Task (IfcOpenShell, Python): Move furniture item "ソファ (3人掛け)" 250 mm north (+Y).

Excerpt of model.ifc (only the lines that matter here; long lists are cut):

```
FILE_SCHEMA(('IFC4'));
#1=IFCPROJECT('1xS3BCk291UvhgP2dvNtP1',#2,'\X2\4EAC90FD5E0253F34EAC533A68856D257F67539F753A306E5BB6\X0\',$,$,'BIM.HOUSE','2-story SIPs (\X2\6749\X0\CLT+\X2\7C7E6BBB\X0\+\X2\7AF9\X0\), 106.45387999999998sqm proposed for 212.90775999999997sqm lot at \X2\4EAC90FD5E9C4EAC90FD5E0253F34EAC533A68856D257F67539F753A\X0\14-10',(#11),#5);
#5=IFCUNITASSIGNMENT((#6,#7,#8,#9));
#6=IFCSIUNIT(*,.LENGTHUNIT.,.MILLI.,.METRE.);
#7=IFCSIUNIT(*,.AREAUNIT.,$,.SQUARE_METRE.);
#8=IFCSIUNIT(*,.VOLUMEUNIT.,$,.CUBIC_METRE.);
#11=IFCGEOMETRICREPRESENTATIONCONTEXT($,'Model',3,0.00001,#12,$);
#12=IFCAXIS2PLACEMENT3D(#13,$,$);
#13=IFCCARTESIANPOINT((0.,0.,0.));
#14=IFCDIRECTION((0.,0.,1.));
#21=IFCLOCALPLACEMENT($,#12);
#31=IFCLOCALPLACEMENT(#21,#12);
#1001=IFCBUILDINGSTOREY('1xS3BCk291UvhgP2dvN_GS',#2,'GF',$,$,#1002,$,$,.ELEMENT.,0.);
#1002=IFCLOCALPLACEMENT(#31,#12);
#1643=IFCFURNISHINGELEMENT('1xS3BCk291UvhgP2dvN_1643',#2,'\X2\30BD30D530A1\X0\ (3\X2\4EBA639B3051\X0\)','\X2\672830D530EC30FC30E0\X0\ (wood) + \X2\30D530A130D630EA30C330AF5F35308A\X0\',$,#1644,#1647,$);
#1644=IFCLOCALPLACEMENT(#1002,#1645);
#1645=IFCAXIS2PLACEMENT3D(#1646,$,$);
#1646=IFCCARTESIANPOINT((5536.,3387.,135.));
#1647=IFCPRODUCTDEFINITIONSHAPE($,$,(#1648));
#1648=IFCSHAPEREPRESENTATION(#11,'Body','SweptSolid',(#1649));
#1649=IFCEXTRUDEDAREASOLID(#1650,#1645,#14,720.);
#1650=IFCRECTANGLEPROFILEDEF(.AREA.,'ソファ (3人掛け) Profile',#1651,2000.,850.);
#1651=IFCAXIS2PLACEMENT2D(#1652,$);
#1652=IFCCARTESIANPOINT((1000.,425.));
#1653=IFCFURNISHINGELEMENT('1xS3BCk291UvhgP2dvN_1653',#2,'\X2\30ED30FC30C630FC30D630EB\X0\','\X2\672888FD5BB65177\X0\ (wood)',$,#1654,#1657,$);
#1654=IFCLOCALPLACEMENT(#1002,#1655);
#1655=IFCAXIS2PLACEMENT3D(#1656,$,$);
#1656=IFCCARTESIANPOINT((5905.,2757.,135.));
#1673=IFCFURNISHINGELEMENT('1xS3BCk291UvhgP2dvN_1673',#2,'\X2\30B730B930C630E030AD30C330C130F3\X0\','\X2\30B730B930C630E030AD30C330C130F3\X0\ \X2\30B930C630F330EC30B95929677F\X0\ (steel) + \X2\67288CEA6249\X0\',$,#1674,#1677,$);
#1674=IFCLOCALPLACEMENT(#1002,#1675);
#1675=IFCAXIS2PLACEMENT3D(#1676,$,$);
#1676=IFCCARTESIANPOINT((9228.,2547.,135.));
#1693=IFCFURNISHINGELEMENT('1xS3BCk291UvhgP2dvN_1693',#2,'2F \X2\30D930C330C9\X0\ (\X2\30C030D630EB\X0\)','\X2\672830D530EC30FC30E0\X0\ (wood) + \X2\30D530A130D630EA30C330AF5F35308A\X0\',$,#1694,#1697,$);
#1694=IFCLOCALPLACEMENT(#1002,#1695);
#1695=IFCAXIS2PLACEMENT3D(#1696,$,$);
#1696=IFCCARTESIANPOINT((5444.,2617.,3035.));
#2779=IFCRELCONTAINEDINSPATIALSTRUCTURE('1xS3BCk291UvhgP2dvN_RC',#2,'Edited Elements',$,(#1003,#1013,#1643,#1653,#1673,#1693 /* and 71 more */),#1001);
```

```python
import ifcopenshell
import ifcopenshell.api.geometry
import ifcopenshell.util.placement

model = ifcopenshell.open("model.ifc")

item = model.by_id(1643)
matrix = ifcopenshell.util.placement.get_local_placement(item.ObjectPlacement)
matrix[1, 3] += 250.0
ifcopenshell.api.geometry.edit_object_placement(model, product=item, matrix=matrix, is_si=False)

print(ifcopenshell.util.placement.get_local_placement(item.ObjectPlacement).round(3) + 0.0)

model.write("model_v2.ifc")
```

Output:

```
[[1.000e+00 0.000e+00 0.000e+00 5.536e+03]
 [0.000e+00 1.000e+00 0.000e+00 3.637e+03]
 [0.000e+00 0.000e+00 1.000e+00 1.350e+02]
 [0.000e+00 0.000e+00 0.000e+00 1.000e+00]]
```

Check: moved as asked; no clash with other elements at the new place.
